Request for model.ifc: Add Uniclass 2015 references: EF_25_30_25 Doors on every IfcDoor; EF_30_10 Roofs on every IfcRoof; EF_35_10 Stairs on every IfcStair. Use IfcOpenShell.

First a look at what the model holds.

```python
import ifcopenshell

model = ifcopenshell.open("model.ifc")
print(model.schema)
print("classifications:", [c.Name for c in model.by_type("IfcClassification")])
for ifc_class in ("IfcDoor", "IfcRoof", "IfcStair", "IfcWall", "IfcWindow"):
    print(ifc_class, len(model.by_type(ifc_class)))
```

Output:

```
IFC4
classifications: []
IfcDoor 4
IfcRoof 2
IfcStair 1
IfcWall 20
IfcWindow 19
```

```python
import ifcopenshell
import ifcopenshell.api.classification

model = ifcopenshell.open("model.ifc")

system = ifcopenshell.api.classification.add_classification(model, classification="Uniclass 2015")

codes = {
    "IfcDoor": ("EF_25_30_25", "Doors"),
    "IfcRoof": ("EF_30_10", "Roofs"),
    "IfcStair": ("EF_35_10", "Stairs"),
}
for ifc_class, (code, name) in codes.items():
    products = model.by_type(ifc_class)
    ifcopenshell.api.classification.add_reference(
        model, products=products, classification=system, identification=code, name=name
    )
    print(code, len(products))

model.write("model_v2.ifc")
```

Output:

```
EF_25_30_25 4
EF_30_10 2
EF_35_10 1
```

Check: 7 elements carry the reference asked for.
